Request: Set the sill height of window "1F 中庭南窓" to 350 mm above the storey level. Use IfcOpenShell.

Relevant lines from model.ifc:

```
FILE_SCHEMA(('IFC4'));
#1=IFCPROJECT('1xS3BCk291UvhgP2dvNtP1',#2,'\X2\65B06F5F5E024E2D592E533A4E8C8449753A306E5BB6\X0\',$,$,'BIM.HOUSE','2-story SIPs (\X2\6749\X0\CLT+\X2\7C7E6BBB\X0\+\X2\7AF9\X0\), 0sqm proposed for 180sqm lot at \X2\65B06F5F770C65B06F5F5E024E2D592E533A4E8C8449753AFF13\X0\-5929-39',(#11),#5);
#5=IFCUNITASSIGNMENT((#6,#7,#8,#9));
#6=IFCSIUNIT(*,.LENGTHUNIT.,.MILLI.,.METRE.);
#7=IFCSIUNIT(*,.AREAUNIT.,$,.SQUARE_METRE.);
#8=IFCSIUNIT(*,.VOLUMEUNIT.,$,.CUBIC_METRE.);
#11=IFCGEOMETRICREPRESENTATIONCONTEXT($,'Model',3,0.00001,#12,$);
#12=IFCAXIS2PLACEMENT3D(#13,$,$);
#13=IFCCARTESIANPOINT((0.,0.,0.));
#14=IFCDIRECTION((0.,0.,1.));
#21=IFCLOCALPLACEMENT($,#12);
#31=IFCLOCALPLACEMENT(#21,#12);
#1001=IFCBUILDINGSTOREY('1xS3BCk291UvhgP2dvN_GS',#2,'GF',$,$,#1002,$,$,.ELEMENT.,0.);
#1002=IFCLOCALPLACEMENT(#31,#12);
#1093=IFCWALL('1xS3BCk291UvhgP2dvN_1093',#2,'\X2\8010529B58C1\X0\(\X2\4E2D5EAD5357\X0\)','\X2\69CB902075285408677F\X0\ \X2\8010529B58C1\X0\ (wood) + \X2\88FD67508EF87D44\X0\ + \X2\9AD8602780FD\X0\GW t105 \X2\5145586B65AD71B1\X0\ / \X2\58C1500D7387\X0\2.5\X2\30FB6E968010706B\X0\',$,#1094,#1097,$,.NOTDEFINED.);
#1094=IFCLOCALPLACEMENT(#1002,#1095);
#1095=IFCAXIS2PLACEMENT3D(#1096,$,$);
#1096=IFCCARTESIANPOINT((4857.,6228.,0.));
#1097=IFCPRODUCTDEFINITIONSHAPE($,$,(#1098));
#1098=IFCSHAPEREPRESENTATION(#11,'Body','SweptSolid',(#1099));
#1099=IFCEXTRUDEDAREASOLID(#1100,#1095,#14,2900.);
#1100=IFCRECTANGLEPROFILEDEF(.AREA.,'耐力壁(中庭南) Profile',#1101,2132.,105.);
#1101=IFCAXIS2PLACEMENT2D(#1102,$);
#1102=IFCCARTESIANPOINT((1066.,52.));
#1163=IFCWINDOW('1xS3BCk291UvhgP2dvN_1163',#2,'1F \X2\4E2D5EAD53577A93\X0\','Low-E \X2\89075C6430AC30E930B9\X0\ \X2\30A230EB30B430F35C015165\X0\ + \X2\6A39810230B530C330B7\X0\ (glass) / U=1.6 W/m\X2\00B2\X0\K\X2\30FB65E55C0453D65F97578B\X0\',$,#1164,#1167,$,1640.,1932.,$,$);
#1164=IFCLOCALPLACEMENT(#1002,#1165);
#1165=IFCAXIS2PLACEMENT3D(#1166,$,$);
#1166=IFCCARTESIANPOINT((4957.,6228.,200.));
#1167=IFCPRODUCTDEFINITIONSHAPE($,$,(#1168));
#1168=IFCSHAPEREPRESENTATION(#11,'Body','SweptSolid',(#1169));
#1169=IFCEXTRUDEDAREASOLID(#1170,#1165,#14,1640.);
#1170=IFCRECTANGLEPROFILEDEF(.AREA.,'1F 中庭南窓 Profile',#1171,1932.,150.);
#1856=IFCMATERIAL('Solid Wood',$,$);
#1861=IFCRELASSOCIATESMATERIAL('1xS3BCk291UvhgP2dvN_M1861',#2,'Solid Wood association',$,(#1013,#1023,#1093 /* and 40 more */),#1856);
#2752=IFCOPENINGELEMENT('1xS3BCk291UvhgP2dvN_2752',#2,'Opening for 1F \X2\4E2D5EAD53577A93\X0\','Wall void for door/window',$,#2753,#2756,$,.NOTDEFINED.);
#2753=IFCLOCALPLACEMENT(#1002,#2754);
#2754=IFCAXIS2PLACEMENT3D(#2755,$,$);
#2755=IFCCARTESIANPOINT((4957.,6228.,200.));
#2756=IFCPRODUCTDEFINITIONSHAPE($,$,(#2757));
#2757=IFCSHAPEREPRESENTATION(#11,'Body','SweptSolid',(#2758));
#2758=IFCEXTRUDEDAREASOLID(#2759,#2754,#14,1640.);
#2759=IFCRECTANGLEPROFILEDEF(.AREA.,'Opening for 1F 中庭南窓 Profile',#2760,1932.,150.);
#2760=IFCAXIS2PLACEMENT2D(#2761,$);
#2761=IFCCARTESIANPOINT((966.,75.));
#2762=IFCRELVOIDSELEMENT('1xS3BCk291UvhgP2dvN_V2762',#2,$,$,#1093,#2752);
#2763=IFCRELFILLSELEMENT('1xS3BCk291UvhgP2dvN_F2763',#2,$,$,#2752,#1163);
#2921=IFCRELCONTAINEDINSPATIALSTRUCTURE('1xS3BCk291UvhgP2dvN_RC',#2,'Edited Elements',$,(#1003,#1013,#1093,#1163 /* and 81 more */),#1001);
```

```python
import numpy as np
import ifcopenshell
import ifcopenshell.api.geometry
import ifcopenshell.geom
import ifcopenshell.util.element
import ifcopenshell.util.placement
import ifcopenshell.util.shape
import ifcopenshell.util.unit

model = ifcopenshell.open("model.ifc")
unit_scale = ifcopenshell.util.unit.calculate_unit_scale(model)

window = model.by_guid("1xS3BCk291UvhgP2dvN_1163")
opening = window.FillsVoids[0].RelatingOpeningElement
storey = ifcopenshell.util.element.get_container(window, ifc_class="IfcBuildingStorey")
level = ifcopenshell.util.placement.get_local_placement(storey.ObjectPlacement)[2, 3]

# The opening's origin need not be at the sill, so measure its lowest point.
shape = ifcopenshell.geom.create_shape(ifcopenshell.geom.settings(), opening)
bottom = ifcopenshell.util.shape.get_shape_bottom_elevation(shape, shape.geometry) / unit_scale
dz = level + 0.35 / unit_scale - bottom

shift = np.array([0.0, 0.0, dz])
# The window is not placed relative to its opening, so move both.
for product in (opening, window):
    matrix = ifcopenshell.util.placement.get_local_placement(product.ObjectPlacement)
    matrix[:3, 3] += shift
    ifcopenshell.api.geometry.edit_object_placement(model, product=product, matrix=matrix, is_si=False)

print(f"moved by {dz * unit_scale:+.3f} m")

model.write("model_updated.ifc")
```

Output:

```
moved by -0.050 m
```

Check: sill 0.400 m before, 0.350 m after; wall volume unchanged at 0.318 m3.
